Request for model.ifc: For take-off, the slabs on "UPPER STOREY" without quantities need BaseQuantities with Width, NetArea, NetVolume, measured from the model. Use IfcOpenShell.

First a look at what the model holds.

```python
import ifcopenshell
import ifcopenshell.util.element
import ifcopenshell.util.unit

model = ifcopenshell.open("model.ifc")
print(model.schema)
for unit_type in ("LENGTHUNIT", "AREAUNIT", "VOLUMEUNIT"):
    print(unit_type, ifcopenshell.util.unit.calculate_unit_scale(model, unit_type))
storey = next(s for s in model.by_type("IfcBuildingStorey") if s.Name == "UPPER STOREY")
slabs = [e for e in ifcopenshell.util.element.get_decomposition(storey) if e.is_a("IfcSlab")]
for e in sorted(slabs, key=lambda e: e.id()):
    print(e.id(), e.is_a(), e.Name, list(ifcopenshell.util.element.get_psets(e, qtos_only=True)), sep=" | ")
```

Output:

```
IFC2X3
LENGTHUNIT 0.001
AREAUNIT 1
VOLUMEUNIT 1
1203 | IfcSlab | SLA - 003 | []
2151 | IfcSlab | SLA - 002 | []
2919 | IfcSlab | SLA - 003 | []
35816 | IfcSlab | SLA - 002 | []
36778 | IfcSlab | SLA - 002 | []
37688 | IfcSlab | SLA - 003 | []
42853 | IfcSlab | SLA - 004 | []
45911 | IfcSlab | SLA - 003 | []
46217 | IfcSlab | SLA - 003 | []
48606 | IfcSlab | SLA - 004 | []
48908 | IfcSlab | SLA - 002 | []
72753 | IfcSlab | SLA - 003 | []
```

```python
import ifcopenshell
import ifcopenshell.api.pset
import ifcopenshell.geom
import ifcopenshell.util.element
import ifcopenshell.util.shape
import ifcopenshell.util.unit

model = ifcopenshell.open("model.ifc")
unit_scale = ifcopenshell.util.unit.calculate_unit_scale(model)
area_scale = ifcopenshell.util.unit.calculate_unit_scale(model, "AREAUNIT")
volume_scale = ifcopenshell.util.unit.calculate_unit_scale(model, "VOLUMEUNIT")
settings = ifcopenshell.geom.settings()

storey = next(s for s in model.by_type("IfcBuildingStorey") if s.Name == "UPPER STOREY")
slabs = [e for e in ifcopenshell.util.element.get_decomposition(storey) if e.is_a("IfcSlab")]

for e in sorted(slabs, key=lambda e: e.id()):
    if ifcopenshell.util.element.get_psets(e, qtos_only=True, should_inherit=False):
        continue
    # Geometry comes back in metres, in the element's own axes.
    shape = ifcopenshell.geom.create_shape(settings, e)
    values = {
        "Width": ifcopenshell.util.shape.get_z(shape.geometry) / unit_scale,
        "NetArea": ifcopenshell.util.shape.get_footprint_area(shape.geometry) / area_scale,
        "NetVolume": ifcopenshell.util.shape.get_volume(shape.geometry) / volume_scale,
    }
    qto = ifcopenshell.api.pset.add_qto(model, product=e, name="BaseQuantities")
    ifcopenshell.api.pset.edit_qto(model, qto=qto, properties=values)
    print(e.id(), {k: round(v, 3) for k, v in values.items()})

model.write("model_updated.ifc")
```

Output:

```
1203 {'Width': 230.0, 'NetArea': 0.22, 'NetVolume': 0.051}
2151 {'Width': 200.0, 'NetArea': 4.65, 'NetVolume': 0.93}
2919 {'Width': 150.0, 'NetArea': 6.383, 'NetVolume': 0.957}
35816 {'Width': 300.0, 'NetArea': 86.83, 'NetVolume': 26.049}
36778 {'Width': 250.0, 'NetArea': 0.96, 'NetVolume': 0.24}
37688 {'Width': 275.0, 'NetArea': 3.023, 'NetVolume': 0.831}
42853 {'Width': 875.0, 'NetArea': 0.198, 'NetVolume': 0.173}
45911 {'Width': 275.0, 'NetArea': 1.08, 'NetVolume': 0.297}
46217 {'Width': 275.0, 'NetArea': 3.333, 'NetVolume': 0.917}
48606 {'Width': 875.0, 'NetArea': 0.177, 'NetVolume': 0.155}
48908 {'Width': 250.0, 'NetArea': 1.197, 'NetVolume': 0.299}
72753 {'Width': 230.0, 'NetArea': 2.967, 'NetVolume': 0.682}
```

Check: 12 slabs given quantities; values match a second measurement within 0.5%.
